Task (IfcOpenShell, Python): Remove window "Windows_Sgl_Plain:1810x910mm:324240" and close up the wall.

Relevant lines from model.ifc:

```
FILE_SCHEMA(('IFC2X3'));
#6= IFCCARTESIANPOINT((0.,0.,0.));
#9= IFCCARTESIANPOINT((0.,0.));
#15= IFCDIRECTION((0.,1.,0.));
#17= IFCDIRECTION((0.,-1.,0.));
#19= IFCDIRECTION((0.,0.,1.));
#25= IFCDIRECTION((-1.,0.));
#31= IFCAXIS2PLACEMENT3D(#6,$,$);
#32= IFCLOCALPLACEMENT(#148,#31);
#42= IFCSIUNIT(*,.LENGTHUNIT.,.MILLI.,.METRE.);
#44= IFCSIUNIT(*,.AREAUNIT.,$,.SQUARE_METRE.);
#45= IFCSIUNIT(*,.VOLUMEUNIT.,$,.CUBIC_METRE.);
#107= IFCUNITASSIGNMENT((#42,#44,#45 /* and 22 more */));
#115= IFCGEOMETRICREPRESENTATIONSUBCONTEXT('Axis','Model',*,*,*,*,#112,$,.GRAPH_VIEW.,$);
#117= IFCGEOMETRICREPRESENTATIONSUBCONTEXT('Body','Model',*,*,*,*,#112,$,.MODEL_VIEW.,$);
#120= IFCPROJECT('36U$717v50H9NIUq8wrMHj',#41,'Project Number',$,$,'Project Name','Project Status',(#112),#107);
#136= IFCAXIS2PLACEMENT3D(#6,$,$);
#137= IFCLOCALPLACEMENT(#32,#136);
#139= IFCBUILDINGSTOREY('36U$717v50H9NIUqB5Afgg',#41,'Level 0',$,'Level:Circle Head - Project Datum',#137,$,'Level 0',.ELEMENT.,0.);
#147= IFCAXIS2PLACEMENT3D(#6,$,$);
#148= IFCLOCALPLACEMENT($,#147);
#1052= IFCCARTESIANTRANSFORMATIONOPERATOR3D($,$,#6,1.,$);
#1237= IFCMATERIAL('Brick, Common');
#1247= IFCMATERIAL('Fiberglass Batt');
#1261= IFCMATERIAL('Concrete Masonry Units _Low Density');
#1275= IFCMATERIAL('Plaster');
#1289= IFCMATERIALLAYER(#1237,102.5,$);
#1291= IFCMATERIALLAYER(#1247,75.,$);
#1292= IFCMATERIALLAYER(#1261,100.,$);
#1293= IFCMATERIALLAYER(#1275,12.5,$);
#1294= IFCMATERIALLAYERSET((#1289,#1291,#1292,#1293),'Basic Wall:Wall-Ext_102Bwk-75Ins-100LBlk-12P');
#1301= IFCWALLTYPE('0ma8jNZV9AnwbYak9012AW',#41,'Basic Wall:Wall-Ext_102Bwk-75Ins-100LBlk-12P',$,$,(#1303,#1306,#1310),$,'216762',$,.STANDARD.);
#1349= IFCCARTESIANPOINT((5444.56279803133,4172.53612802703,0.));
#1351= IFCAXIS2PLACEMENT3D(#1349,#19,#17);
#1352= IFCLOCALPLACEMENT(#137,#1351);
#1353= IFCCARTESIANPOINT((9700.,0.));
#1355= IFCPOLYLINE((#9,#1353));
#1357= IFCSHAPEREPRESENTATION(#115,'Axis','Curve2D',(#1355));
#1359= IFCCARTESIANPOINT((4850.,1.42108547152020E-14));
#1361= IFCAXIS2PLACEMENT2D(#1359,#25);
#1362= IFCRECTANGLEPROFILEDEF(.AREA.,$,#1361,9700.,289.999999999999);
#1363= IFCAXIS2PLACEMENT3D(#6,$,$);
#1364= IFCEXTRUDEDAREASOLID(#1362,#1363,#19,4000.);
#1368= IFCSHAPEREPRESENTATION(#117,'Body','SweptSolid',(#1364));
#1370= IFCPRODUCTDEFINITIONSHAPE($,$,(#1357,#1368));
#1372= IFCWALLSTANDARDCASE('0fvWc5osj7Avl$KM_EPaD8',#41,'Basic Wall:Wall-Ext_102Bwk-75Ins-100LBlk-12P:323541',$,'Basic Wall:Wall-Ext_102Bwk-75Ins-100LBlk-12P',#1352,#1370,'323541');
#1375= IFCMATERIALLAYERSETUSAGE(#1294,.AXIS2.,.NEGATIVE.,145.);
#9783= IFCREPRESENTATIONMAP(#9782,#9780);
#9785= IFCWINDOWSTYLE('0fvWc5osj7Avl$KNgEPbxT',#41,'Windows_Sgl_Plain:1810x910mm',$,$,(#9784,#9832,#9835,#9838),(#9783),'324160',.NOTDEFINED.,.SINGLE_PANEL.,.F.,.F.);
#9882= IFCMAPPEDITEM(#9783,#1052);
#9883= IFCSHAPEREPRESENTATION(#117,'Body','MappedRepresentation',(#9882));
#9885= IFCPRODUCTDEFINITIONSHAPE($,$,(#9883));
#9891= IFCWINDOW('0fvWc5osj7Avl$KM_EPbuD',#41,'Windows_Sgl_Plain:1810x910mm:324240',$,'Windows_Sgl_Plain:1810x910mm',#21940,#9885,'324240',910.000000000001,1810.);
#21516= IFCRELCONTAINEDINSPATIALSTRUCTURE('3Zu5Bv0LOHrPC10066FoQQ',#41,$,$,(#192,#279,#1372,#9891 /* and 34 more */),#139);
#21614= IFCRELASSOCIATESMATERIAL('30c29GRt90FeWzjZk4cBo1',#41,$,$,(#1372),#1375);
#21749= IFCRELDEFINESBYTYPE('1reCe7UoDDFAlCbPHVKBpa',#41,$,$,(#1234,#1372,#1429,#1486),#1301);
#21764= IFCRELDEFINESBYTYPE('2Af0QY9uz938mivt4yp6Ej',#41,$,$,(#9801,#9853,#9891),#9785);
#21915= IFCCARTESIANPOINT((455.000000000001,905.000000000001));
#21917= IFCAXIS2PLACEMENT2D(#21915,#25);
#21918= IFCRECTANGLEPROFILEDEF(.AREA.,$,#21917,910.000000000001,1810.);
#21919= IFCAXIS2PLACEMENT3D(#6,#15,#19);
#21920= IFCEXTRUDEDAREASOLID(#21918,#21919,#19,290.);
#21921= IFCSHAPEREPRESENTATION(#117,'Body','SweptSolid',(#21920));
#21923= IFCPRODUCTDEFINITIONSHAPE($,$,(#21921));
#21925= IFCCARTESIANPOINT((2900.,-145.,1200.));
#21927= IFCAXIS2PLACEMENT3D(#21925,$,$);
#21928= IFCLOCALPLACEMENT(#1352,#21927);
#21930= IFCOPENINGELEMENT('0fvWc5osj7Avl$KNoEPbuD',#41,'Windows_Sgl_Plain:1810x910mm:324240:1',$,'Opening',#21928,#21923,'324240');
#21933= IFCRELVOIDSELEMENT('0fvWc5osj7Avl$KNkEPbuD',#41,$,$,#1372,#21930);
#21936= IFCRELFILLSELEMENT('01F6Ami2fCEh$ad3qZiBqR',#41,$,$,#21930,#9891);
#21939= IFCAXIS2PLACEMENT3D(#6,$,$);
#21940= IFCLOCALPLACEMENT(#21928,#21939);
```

```python
import ifcopenshell
import ifcopenshell.api.feature
import ifcopenshell.api.root
import ifcopenshell.geom
import ifcopenshell.util.shape

model = ifcopenshell.open("model.ifc")
settings = ifcopenshell.geom.settings()


def volume(element):
    """Net volume in cubic metres, openings subtracted."""
    shape = ifcopenshell.geom.create_shape(settings, element)
    return ifcopenshell.util.shape.get_volume(shape.geometry)


window = model.by_guid("0fvWc5osj7Avl$KM_EPbuD")
opening = window.FillsVoids[0].RelatingOpeningElement
wall = opening.VoidsElements[0].RelatingBuildingElement
before = volume(wall)

ifcopenshell.api.root.remove_product(model, product=window)
ifcopenshell.api.feature.remove_feature(model, feature=opening)

after = volume(wall)

print(f"wall volume {before:.3f} -> {after:.3f} m3")

model.write("model-out.ifc")
```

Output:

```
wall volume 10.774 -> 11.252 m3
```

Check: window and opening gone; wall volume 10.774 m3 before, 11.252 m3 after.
